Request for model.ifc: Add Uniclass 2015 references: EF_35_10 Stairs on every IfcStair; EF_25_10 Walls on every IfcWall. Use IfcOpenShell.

First a look at what the model holds.

```python
import ifcopenshell

model = ifcopenshell.open("model.ifc")
print(model.schema)
print("classifications:", [c.Name for c in model.by_type("IfcClassification")])
for ifc_class in ("IfcDoor", "IfcRoof", "IfcStair", "IfcWall", "IfcWindow"):
    print(ifc_class, len(model.by_type(ifc_class)))
```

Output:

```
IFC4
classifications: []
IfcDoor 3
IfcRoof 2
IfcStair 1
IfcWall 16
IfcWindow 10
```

```python
import ifcopenshell
import ifcopenshell.api.classification

model = ifcopenshell.open("model.ifc")

system = ifcopenshell.api.classification.add_classification(model, classification="Uniclass 2015")

codes = {
    "IfcStair": ("EF_35_10", "Stairs"),
    "IfcWall": ("EF_25_10", "Walls"),
}
for ifc_class, (code, name) in codes.items():
    products = model.by_type(ifc_class)
    ifcopenshell.api.classification.add_reference(
        model, products=products, classification=system, identification=code, name=name
    )
    print(code, len(products))

model.write("model_updated.ifc")
```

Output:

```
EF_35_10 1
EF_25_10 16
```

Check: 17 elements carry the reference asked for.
